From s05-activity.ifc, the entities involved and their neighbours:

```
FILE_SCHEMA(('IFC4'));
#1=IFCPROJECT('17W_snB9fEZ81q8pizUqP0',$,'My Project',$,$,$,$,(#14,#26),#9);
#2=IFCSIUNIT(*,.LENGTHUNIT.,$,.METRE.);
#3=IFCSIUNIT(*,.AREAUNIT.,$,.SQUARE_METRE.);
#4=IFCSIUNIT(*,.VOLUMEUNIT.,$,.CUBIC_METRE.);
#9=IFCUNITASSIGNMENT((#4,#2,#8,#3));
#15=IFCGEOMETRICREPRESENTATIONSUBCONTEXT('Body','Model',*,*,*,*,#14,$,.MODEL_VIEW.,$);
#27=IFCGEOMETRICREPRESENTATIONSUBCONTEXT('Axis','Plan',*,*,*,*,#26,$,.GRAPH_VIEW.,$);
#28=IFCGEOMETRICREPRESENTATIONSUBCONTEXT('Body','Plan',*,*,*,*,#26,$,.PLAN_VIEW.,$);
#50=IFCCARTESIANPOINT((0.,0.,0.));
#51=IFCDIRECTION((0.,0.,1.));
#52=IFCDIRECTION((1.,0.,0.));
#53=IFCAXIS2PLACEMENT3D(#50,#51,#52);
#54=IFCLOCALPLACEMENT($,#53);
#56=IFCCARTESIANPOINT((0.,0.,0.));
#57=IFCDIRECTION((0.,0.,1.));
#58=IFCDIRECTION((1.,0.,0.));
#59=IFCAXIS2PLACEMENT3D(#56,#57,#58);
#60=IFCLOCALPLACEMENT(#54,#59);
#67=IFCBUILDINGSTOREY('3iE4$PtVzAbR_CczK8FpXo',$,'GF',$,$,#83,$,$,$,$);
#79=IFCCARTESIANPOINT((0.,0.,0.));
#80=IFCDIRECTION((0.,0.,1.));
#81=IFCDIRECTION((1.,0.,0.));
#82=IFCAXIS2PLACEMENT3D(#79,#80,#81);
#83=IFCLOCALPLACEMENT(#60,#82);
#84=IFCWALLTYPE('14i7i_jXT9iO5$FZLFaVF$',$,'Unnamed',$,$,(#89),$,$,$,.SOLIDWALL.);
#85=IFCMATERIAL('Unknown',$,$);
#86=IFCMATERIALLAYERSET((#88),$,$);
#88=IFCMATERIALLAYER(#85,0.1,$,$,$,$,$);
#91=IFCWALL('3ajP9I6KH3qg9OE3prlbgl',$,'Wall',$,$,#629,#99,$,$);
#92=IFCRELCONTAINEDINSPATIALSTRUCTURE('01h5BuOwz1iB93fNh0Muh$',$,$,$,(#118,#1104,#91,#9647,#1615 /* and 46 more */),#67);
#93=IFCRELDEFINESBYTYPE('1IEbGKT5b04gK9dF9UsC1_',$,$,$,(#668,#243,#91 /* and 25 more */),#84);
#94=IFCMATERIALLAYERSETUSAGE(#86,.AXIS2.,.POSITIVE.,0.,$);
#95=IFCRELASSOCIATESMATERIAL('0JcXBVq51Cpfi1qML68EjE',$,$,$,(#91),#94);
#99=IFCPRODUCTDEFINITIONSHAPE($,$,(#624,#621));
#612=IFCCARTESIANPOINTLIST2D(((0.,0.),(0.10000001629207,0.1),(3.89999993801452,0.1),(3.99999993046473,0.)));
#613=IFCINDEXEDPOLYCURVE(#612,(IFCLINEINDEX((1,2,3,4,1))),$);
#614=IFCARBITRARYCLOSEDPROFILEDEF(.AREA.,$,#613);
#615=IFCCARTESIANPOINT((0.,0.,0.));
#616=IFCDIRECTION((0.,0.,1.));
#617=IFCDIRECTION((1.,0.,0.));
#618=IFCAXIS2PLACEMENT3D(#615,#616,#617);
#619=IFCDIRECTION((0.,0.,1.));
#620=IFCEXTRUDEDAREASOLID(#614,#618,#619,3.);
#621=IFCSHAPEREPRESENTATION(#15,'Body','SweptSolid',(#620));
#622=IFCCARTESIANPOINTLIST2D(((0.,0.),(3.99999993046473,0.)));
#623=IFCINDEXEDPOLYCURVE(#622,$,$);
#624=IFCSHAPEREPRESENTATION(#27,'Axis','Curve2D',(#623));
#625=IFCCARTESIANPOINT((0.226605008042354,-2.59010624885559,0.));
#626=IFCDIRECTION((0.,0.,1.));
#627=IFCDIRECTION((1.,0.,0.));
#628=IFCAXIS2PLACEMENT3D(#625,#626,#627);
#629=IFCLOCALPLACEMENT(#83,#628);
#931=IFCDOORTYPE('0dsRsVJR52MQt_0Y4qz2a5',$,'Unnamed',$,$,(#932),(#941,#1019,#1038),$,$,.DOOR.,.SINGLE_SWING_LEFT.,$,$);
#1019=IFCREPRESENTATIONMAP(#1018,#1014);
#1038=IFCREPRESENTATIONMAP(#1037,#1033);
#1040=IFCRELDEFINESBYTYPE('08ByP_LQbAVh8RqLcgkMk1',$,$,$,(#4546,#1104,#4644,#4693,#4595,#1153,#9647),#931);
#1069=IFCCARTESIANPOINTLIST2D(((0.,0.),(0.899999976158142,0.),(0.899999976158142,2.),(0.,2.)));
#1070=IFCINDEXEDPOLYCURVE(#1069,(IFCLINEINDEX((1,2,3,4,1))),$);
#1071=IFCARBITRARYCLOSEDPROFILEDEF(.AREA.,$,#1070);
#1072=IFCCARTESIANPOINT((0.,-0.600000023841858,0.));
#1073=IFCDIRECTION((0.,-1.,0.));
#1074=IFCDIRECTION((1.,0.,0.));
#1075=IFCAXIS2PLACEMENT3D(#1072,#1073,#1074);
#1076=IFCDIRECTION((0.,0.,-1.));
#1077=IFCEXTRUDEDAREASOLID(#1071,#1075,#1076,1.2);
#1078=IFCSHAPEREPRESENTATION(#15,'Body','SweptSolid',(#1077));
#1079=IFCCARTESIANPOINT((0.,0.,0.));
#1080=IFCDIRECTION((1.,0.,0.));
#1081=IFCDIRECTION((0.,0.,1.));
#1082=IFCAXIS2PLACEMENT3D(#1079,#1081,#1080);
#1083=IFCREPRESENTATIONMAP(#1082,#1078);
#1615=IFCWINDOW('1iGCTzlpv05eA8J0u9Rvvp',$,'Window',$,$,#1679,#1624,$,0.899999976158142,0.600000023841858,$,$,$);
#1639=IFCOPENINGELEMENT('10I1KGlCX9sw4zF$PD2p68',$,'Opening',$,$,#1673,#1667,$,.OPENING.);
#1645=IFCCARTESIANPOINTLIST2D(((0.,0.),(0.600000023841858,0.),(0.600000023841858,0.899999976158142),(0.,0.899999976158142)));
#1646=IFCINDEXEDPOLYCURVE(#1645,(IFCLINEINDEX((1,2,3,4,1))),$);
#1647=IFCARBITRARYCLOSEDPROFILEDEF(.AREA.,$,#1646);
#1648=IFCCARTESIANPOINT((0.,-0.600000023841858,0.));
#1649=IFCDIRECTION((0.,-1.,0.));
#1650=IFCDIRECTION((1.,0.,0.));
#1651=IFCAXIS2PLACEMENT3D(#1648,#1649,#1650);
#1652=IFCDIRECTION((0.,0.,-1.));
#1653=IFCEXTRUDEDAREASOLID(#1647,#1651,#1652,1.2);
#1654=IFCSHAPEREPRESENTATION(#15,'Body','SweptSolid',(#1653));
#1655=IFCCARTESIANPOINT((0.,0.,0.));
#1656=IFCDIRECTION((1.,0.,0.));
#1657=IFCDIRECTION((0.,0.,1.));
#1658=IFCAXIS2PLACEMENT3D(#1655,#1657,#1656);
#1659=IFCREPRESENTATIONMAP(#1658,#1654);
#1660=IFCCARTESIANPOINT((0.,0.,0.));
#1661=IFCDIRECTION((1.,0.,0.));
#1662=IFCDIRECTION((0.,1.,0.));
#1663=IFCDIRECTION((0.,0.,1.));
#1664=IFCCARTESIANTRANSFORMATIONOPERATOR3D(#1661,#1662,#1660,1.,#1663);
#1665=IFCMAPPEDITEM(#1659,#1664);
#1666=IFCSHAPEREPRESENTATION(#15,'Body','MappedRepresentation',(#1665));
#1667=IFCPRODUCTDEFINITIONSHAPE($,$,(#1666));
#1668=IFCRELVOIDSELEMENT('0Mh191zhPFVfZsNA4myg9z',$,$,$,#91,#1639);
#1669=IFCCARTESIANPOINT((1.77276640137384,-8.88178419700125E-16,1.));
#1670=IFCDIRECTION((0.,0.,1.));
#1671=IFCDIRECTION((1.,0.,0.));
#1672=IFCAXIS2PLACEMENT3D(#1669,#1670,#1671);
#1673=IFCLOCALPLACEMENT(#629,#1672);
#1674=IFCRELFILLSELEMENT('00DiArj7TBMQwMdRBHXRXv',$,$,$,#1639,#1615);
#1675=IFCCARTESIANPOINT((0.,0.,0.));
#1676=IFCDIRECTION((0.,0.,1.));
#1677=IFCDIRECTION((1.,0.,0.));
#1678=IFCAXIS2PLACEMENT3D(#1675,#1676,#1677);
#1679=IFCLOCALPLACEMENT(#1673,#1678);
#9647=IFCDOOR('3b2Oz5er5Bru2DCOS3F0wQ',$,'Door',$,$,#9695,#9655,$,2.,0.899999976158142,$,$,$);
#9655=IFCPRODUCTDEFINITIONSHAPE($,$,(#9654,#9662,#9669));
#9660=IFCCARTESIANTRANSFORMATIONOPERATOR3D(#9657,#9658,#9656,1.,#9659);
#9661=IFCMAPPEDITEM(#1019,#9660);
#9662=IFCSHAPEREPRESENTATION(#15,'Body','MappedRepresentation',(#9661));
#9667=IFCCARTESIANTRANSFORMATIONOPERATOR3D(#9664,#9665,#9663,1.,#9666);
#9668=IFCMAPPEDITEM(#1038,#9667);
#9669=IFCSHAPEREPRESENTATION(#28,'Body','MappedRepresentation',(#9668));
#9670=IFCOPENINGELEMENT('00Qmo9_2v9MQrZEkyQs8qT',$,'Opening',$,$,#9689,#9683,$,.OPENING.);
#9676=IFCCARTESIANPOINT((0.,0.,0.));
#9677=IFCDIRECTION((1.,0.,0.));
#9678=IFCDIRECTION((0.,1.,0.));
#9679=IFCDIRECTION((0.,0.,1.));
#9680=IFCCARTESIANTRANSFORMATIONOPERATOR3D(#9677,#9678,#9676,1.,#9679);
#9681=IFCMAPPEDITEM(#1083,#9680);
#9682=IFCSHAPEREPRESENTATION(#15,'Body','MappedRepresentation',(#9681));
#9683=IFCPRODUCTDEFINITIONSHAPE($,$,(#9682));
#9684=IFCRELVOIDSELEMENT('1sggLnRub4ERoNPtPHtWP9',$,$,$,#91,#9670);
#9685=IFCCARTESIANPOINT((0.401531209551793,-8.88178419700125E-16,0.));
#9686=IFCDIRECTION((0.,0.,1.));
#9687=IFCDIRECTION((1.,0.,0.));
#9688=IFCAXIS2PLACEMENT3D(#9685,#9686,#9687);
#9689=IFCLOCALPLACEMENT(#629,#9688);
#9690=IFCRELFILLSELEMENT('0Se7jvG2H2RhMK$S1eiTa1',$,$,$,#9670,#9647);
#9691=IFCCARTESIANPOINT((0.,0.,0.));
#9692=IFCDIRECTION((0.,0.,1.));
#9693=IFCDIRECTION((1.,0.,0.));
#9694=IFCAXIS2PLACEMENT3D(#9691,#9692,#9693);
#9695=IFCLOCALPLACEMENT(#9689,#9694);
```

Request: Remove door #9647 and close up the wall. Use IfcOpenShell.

```python
import ifcopenshell
import ifcopenshell.api.feature
import ifcopenshell.api.root
import ifcopenshell.geom
import ifcopenshell.util.shape

model = ifcopenshell.open("s05-activity.ifc")
settings = ifcopenshell.geom.settings()


def volume(element):
    """Net volume in cubic metres, openings subtracted."""
    shape = ifcopenshell.geom.create_shape(settings, element)
    return ifcopenshell.util.shape.get_volume(shape.geometry)


door = model.by_guid("3b2Oz5er5Bru2DCOS3F0wQ")
opening = door.FillsVoids[0].RelatingOpeningElement
wall = opening.VoidsElements[0].RelatingBuildingElement
before = volume(wall)

ifcopenshell.api.root.remove_product(model, product=door)
ifcopenshell.api.feature.remove_feature(model, feature=opening)

after = volume(wall)

print(f"wall volume {before:.3f} -> {after:.3f} m3")

model.write("s05-activity_rev.ifc")
```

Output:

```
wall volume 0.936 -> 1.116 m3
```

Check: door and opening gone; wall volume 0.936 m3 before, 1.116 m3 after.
